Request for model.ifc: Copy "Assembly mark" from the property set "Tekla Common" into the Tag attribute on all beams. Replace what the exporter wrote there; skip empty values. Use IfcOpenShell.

First a look at what the model holds.

```python
import ifcopenshell
import ifcopenshell.util.element

model = ifcopenshell.open("model.ifc")
print(model.schema)
beams = model.by_type("IfcBeam")
print(len(beams), "beams")
for e in beams[:8]:
    source = ifcopenshell.util.element.get_pset(e, "Tekla Common", "Assembly mark")
    target = e.Tag
    print(e.id(), repr(source), repr(target), sep=" | ")
```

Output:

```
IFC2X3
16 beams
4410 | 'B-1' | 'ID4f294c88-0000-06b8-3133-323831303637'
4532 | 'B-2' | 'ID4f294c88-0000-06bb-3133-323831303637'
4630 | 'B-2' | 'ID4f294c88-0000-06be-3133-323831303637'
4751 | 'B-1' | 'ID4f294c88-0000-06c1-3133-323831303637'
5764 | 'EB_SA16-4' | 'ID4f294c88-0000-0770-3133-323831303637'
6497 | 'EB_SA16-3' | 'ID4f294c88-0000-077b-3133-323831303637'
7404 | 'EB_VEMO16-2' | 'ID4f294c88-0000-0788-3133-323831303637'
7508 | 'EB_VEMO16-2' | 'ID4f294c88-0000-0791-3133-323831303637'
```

```python
import ifcopenshell
import ifcopenshell.util.element

model = ifcopenshell.open("model.ifc")

count = 0
for e in model.by_type("IfcBeam"):
    value = ifcopenshell.util.element.get_pset(e, "Tekla Common", "Assembly mark")
    current = e.Tag
    if not value or not value.strip() or current == value:
        continue
    e.Tag = value
    count += 1

print(count, "beams updated")

model.write("model_updated.ifc")
```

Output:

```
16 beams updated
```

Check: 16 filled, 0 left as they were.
